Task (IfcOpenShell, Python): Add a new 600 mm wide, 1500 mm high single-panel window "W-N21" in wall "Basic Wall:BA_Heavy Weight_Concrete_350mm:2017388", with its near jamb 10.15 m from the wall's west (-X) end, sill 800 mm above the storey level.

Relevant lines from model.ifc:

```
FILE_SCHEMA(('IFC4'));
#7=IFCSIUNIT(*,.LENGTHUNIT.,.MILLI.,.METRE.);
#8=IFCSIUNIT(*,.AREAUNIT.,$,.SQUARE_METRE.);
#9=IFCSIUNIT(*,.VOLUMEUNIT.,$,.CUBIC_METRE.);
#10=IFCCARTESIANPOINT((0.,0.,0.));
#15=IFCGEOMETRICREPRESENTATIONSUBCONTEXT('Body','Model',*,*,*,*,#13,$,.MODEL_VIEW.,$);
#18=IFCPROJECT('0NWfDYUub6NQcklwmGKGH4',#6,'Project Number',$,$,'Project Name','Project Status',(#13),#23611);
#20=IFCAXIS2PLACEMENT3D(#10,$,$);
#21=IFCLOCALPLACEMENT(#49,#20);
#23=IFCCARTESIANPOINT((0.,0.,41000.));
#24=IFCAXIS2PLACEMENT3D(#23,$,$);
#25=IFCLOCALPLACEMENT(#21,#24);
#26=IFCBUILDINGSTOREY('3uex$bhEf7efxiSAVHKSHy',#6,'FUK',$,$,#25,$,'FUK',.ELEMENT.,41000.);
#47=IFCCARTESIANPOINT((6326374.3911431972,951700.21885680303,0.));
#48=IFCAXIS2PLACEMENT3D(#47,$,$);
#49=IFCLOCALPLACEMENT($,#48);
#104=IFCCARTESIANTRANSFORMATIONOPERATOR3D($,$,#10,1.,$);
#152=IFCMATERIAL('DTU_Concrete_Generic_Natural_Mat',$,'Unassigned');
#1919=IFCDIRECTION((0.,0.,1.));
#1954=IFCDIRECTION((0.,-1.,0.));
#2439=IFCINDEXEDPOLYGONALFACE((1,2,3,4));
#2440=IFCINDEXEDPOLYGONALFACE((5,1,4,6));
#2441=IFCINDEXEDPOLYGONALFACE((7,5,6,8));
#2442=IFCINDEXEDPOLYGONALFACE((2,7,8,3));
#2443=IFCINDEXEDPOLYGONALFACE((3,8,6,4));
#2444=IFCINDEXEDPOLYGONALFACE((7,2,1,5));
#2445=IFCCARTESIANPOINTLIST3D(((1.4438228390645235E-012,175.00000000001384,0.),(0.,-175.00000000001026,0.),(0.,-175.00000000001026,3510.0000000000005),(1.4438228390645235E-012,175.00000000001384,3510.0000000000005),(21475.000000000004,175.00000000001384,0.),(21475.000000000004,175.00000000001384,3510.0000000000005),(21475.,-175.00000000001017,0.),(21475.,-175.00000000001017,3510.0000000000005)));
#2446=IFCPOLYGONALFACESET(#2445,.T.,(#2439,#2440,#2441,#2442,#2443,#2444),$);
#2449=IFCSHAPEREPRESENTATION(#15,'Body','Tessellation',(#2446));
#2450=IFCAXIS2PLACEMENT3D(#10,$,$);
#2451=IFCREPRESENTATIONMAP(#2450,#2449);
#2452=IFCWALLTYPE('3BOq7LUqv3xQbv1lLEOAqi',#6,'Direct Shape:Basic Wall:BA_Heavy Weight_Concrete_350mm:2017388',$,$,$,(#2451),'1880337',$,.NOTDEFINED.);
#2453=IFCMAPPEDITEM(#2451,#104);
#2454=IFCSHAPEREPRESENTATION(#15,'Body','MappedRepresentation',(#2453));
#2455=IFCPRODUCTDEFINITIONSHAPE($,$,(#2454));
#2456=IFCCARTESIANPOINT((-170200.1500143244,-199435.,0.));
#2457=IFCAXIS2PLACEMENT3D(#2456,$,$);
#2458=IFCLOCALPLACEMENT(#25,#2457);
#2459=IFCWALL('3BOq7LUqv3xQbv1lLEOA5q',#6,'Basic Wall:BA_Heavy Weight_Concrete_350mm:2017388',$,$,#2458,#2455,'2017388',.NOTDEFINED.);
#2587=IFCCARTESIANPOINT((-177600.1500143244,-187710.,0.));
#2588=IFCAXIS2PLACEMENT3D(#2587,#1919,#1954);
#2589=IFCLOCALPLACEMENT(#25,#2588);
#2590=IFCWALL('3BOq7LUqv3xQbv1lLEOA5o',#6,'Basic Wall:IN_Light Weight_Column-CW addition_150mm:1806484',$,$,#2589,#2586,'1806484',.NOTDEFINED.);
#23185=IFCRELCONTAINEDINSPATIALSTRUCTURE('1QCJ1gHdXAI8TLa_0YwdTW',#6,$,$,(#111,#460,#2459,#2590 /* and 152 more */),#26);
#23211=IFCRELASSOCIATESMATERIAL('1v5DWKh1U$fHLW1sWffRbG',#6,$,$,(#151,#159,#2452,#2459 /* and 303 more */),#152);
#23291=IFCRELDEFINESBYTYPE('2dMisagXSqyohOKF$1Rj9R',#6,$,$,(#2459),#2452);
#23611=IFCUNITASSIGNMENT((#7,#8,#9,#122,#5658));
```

```python
import numpy as np
import ifcopenshell
import ifcopenshell.api.feature
import ifcopenshell.api.geometry
import ifcopenshell.api.root
import ifcopenshell.api.spatial
import ifcopenshell.geom
import ifcopenshell.util.element
import ifcopenshell.util.placement
import ifcopenshell.util.representation
import ifcopenshell.util.shape
import ifcopenshell.util.unit

model = ifcopenshell.open("model.ifc")
unit_scale = ifcopenshell.util.unit.calculate_unit_scale(model)
settings = ifcopenshell.geom.settings()


def volume(element):
    """Net volume in cubic metres, openings subtracted."""
    shape = ifcopenshell.geom.create_shape(settings, element)
    return ifcopenshell.util.shape.get_volume(shape.geometry)


wall = model.by_guid("3BOq7LUqv3xQbv1lLEOA5q")
storey = ifcopenshell.util.element.get_container(wall, ifc_class="IfcBuildingStorey")
context = ifcopenshell.util.representation.get_context(model, "Model", "Body", "MODEL_VIEW")
before = volume(wall)

width, height, from_end, sill = 0.6, 1.5, 10.15, 0.8  # metres

# The wall runs along its own X axis, and the end named is its -X end.
wall_shape = ifcopenshell.geom.create_shape(settings, wall)
x, y, z = ifcopenshell.util.shape.get_vertices(wall_shape.geometry).T
start = x.min() + from_end
face, thickness = float(y.min()), float(y.max() - y.min())
wall_matrix = ifcopenshell.util.placement.get_local_placement(wall.ObjectPlacement)
level = ifcopenshell.util.placement.get_local_placement(storey.ObjectPlacement)[2, 3]


def in_wall(x, y):
    """Placement at x, y metres in the wall's axes, at sill height."""
    matrix = wall_matrix.copy()
    matrix[:, 3] = wall_matrix @ np.array([x / unit_scale, y / unit_scale, 0.0, 1.0])
    matrix[2, 3] = level + sill / unit_scale
    return matrix


# Opening: a box that overshoots both wall faces by 50 mm.
opening = ifcopenshell.api.root.create_entity(model, ifc_class="IfcOpeningElement", predefined_type="OPENING")
box = ifcopenshell.api.geometry.add_wall_representation(
    model, context=context, length=width, height=height, thickness=thickness + 0.1
)
ifcopenshell.api.geometry.assign_representation(model, product=opening, representation=box)
ifcopenshell.api.geometry.edit_object_placement(model, product=opening, matrix=in_wall(start, face - 0.05), is_si=False)
ifcopenshell.api.feature.add_feature(model, feature=opening, element=wall)

window = ifcopenshell.api.root.create_entity(model, ifc_class="IfcWindow", name="W-N21", predefined_type="WINDOW")
window.OverallWidth, window.OverallHeight = width / unit_scale, height / unit_scale
window.PartitioningType = "SINGLE_PANEL"
body = ifcopenshell.api.geometry.add_window_representation(
    model,
    context=context,
    overall_width=window.OverallWidth,
    overall_height=window.OverallHeight,
    partition_type="SINGLE_PANEL",
)
ifcopenshell.api.geometry.assign_representation(model, product=window, representation=body)
ifcopenshell.api.spatial.assign_container(model, products=[window], relating_structure=storey)
ifcopenshell.api.feature.add_filling(model, opening=opening, element=window)

# Centre the window in the wall's thickness.
ifcopenshell.api.geometry.edit_object_placement(model, product=window, matrix=in_wall(start, face), is_si=False)
window_shape = ifcopenshell.geom.create_shape(settings, window)
depth = ifcopenshell.util.shape.get_vertices(window_shape.geometry)[:, 1]
offset = face + thickness / 2 - (depth.min() + depth.max()) / 2
ifcopenshell.api.geometry.edit_object_placement(model, product=window, matrix=in_wall(start, offset), is_si=False)

after = volume(wall)

print(f"wall volume {before:.3f} -> {after:.3f} m3")

model.write("model_v2.ifc")
```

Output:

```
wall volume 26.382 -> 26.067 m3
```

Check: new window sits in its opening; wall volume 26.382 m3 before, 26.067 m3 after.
